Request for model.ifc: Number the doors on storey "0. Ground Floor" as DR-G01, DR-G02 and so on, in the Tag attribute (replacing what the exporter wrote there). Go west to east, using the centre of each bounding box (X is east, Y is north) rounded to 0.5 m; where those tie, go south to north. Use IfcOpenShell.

First a look at what the model holds.

```python
import ifcopenshell
import ifcopenshell.util.element
import ifcopenshell.util.placement

model = ifcopenshell.open("model.ifc")
print(model.schema)
storey = next(s for s in model.by_type("IfcBuildingStorey") if s.Name == "0. Ground Floor")
doors = [e for e in ifcopenshell.util.element.get_decomposition(storey) if e.is_a("IfcDoor")]
for e in sorted(doors, key=lambda e: e.id()):
    origin = ifcopenshell.util.placement.get_local_placement(e.ObjectPlacement)[:3, 3]
    print(e.id(), e.Tag, e.Name, origin.round(2) + 0.0, sep=" | ")
```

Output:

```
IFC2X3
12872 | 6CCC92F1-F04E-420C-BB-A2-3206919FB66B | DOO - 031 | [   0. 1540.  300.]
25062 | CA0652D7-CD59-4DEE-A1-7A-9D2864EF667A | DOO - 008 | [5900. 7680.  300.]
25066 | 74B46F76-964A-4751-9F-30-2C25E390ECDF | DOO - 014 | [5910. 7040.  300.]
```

```python
import ifcopenshell
import ifcopenshell.geom
import ifcopenshell.util.element
import ifcopenshell.util.shape

model = ifcopenshell.open("model.ifc")
settings = ifcopenshell.geom.settings()
settings.set("use-world-coords", True)


def centre(element):
    shape = ifcopenshell.geom.create_shape(settings, element)
    return ifcopenshell.util.shape.get_bbox_centroid(shape.geometry)


storey = next(s for s in model.by_type("IfcBuildingStorey") if s.Name == "0. Ground Floor")
doors = [e for e in ifcopenshell.util.element.get_decomposition(storey) if e.is_a("IfcDoor")]

# Insertion points can sit at a corner or the storey origin, so sort by the geometry (in metres).
centres = {e: centre(e) for e in doors}
doors.sort(key=lambda e: (round(centres[e][0] / 0.5), centres[e][1]))

for i, e in enumerate(doors, start=1):
    number = f"DR-G{i:02d}"
    e.Tag = number
    print(e.id(), number)

model.write("model_edited.ifc")
```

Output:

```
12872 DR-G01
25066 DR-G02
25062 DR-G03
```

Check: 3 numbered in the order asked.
